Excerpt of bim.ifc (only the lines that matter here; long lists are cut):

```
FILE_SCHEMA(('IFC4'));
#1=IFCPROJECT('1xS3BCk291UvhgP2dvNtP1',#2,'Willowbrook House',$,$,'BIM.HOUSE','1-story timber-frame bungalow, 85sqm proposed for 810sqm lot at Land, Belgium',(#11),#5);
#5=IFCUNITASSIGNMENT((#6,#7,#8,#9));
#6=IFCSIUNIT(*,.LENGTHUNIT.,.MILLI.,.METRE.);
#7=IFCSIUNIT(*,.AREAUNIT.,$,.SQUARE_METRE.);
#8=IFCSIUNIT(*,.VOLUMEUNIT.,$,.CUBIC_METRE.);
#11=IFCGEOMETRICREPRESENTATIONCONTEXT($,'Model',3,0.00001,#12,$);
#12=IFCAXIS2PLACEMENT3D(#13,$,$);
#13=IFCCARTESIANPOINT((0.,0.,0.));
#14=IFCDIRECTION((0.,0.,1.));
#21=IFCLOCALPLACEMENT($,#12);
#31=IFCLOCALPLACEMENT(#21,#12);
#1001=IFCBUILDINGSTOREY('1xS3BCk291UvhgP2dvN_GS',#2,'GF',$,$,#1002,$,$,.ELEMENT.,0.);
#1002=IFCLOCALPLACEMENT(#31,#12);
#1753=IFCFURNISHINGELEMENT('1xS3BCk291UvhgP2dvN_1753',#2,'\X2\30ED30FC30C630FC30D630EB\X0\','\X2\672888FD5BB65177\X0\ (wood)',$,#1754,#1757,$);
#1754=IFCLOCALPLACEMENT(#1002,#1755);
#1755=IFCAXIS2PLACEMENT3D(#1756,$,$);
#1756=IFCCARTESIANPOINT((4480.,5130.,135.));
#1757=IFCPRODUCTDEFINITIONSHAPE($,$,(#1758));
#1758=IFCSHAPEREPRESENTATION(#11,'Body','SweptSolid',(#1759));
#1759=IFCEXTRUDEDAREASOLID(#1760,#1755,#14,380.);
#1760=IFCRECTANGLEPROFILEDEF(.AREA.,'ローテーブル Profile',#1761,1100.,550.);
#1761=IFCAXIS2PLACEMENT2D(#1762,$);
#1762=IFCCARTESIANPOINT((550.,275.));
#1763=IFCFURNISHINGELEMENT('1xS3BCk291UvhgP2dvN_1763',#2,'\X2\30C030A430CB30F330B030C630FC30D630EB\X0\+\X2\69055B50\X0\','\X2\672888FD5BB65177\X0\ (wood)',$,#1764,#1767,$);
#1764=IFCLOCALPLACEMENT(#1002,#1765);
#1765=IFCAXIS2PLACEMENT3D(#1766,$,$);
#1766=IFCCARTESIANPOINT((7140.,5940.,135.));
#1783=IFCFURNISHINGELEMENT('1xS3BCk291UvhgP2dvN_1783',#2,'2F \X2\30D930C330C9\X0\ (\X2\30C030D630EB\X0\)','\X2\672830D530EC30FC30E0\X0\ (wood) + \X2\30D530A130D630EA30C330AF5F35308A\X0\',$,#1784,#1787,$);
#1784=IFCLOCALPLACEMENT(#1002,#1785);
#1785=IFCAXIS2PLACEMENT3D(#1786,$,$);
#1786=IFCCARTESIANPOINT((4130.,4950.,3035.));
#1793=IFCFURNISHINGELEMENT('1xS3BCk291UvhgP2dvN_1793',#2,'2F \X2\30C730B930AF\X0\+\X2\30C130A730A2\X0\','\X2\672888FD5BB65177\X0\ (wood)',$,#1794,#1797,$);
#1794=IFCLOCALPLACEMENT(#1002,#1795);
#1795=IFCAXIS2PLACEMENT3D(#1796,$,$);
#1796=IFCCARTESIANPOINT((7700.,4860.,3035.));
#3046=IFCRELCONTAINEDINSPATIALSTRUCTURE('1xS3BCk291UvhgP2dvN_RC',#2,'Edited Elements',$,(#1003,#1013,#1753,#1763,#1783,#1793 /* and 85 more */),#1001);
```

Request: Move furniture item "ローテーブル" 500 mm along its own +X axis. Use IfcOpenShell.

```python
import ifcopenshell
import ifcopenshell.api.geometry
import ifcopenshell.util.placement
import ifcopenshell.util.unit

model = ifcopenshell.open("bim.ifc")
unit_scale = ifcopenshell.util.unit.calculate_unit_scale(model)

item = model.by_guid("1xS3BCk291UvhgP2dvN_1753")
matrix = ifcopenshell.util.placement.get_local_placement(item.ObjectPlacement)
matrix[:3, 3] += matrix[:3, 0] * 0.5 / unit_scale
ifcopenshell.api.geometry.edit_object_placement(model, product=item, matrix=matrix, is_si=False)

print(ifcopenshell.util.placement.get_local_placement(item.ObjectPlacement).round(3) + 0.0)

model.write("bim_rev.ifc")
```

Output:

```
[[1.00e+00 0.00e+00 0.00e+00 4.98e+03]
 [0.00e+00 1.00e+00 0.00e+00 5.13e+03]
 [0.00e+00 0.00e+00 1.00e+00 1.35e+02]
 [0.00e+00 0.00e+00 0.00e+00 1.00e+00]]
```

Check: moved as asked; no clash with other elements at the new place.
